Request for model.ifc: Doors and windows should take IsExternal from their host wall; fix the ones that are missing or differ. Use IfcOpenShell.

First a look at what the model holds.

```python
import ifcopenshell
import ifcopenshell.util.element

model = ifcopenshell.open("model.ifc")
print(model.schema)
seen = {}
for e in model.by_type("IfcDoor") + model.by_type("IfcWindow"):
    if not e.FillsVoids:
        continue
    host = e.FillsVoids[0].RelatingOpeningElement.VoidsElements[0].RelatingBuildingElement
    own = ifcopenshell.util.element.get_pset(e, f"Pset_{e.is_a()[3:].removesuffix('StandardCase')}Common", "IsExternal")
    wall = ifcopenshell.util.element.get_pset(host, "Pset_WallCommon", "IsExternal")
    seen[e.is_a(), own, wall] = seen.get((e.is_a(), own, wall), 0) + 1
for (cls, own, wall), count in sorted(seen.items(), key=str):
    print(count, cls, "IsExternal:", own, "| host wall:", wall)
```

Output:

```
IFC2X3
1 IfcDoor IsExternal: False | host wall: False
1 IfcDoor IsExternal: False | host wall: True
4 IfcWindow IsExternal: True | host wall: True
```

```python
import ifcopenshell
import ifcopenshell.api.pset
import ifcopenshell.util.element

model = ifcopenshell.open("model.ifc")

count = 0
for ifc_class, pset_name in (("IfcDoor", "Pset_DoorCommon"), ("IfcWindow", "Pset_WindowCommon")):
    for e in model.by_type(ifc_class):
        if not e.FillsVoids:
            continue
        host = e.FillsVoids[0].RelatingOpeningElement.VoidsElements[0].RelatingBuildingElement
        external = ifcopenshell.util.element.get_pset(host, "Pset_WallCommon", "IsExternal")
        if external is None or ifcopenshell.util.element.get_pset(e, pset_name, "IsExternal") == external:
            continue
        pset = ifcopenshell.api.pset.add_pset(model, product=e, name=pset_name)
        ifcopenshell.api.pset.edit_pset(model, pset=pset, properties={"IsExternal": external})
        count += 1

print(count, "updated")

model.write("model_rev.ifc")
```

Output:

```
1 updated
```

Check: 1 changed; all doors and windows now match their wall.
